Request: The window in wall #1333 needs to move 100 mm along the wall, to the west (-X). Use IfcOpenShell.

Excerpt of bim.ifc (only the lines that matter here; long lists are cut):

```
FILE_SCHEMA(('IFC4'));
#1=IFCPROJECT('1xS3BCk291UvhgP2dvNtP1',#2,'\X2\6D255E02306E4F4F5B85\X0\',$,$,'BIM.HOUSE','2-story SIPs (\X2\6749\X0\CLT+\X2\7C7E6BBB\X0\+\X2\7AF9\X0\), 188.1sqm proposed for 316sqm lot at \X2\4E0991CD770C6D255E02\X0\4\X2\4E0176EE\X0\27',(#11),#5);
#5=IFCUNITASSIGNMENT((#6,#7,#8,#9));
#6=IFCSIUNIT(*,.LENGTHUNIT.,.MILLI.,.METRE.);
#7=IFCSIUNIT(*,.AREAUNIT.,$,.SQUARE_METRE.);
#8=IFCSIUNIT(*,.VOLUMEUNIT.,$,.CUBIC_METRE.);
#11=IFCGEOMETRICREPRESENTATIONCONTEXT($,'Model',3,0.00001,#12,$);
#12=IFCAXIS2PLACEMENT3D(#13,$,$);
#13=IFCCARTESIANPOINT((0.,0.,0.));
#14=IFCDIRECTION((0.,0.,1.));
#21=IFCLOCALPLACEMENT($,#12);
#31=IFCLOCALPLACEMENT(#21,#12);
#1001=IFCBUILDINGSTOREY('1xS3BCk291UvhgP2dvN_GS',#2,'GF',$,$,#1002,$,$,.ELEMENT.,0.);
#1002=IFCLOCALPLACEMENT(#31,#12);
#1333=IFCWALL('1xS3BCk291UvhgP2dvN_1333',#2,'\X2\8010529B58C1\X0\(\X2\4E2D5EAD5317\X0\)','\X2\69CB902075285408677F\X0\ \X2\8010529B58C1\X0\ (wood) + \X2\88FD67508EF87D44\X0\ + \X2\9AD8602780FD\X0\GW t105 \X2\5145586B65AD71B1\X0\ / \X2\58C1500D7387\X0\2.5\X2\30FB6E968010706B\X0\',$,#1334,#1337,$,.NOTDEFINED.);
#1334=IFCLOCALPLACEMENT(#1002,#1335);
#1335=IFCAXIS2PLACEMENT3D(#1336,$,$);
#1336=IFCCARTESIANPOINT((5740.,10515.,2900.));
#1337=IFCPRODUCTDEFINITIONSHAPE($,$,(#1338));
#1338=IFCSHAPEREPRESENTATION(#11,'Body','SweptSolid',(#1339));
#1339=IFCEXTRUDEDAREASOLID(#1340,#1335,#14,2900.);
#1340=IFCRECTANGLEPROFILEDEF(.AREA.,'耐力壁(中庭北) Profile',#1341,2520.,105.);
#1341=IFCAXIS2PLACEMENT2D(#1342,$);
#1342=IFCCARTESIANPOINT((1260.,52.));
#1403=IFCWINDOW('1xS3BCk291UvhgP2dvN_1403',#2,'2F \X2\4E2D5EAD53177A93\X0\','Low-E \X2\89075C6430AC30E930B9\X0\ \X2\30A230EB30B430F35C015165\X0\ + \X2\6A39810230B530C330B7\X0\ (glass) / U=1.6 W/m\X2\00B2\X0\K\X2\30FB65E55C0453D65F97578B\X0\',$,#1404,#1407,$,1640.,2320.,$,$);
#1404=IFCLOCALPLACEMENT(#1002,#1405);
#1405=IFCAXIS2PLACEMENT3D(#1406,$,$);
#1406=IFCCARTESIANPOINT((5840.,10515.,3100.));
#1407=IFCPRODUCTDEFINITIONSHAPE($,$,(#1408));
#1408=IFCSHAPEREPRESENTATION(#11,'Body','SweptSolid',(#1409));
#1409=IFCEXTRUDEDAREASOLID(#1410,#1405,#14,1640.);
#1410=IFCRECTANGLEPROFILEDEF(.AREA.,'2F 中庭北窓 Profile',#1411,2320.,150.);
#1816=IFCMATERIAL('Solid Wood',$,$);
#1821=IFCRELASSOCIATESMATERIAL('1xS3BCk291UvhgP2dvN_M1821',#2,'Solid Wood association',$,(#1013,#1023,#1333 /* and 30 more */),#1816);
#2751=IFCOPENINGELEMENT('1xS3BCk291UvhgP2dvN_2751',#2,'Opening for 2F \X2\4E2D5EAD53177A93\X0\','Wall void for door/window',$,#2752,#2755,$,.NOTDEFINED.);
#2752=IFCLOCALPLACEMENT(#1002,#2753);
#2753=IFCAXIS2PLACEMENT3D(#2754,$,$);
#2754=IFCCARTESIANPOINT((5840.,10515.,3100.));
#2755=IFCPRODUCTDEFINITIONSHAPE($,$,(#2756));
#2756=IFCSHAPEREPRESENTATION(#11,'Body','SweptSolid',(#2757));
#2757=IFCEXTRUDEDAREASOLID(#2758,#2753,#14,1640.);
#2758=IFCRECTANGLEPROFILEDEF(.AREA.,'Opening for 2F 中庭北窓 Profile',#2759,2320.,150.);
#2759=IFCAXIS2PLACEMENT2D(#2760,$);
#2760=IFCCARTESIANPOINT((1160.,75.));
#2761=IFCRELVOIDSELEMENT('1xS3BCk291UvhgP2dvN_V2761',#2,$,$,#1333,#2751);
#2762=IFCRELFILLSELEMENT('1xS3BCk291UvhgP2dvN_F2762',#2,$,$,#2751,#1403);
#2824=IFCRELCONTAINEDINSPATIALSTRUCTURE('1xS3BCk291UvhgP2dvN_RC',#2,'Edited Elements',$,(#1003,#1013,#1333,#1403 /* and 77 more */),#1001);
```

```python
import ifcopenshell
import ifcopenshell.api.geometry
import ifcopenshell.util.placement
import ifcopenshell.util.unit

model = ifcopenshell.open("bim.ifc")
unit_scale = ifcopenshell.util.unit.calculate_unit_scale(model)

window = model.by_id(1403)
opening = window.FillsVoids[0].RelatingOpeningElement
wall = opening.VoidsElements[0].RelatingBuildingElement

wall_matrix = ifcopenshell.util.placement.get_local_placement(wall.ObjectPlacement)
shift = wall_matrix[:3, 0] * -0.1 / unit_scale
before = ifcopenshell.util.placement.get_local_placement(window.ObjectPlacement)[:3, 3].copy()

# The window is not placed relative to its opening, so move both.
for product in (opening, window):
    matrix = ifcopenshell.util.placement.get_local_placement(product.ObjectPlacement)
    matrix[:3, 3] += shift
    ifcopenshell.api.geometry.edit_object_placement(model, product=product, matrix=matrix, is_si=False)

after = ifcopenshell.util.placement.get_local_placement(window.ObjectPlacement)[:3, 3]
print("window moved by", (after - before).round(3) + 0.0)

model.write("bim_rev.ifc")
```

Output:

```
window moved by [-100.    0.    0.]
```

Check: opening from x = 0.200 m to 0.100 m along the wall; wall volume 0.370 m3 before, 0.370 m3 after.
